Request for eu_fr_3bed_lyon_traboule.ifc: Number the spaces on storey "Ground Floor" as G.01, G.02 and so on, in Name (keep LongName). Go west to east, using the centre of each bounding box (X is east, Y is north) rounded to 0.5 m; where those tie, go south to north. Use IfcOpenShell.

First a look at what the model holds.

```python
import ifcopenshell
import ifcopenshell.util.element
import ifcopenshell.util.placement

model = ifcopenshell.open("eu_fr_3bed_lyon_traboule.ifc")
print(model.schema)
storey = next(s for s in model.by_type("IfcBuildingStorey") if s.Name == "Ground Floor")
spaces = [e for e in ifcopenshell.util.element.get_decomposition(storey) if e.is_a("IfcSpace")]
for e in sorted(spaces, key=lambda e: e.id()):
    origin = ifcopenshell.util.placement.get_local_placement(e.ObjectPlacement)[:3, 3]
    print(e.id(), e.Name, e.LongName, origin.round(2) + 0.0, sep=" | ")
```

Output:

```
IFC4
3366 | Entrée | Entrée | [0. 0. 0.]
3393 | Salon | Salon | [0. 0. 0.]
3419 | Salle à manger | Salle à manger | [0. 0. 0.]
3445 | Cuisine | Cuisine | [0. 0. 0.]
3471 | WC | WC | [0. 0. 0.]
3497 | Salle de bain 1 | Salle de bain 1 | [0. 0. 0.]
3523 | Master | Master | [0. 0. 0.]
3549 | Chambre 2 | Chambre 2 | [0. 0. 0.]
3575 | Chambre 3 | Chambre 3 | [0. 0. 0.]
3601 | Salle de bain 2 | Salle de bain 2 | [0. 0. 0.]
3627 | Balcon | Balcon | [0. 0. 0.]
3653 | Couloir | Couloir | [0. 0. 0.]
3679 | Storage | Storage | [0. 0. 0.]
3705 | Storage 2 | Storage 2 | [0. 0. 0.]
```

```python
import ifcopenshell
import ifcopenshell.geom
import ifcopenshell.util.element
import ifcopenshell.util.shape

model = ifcopenshell.open("eu_fr_3bed_lyon_traboule.ifc")
settings = ifcopenshell.geom.settings()
settings.set("use-world-coords", True)


def centre(element):
    shape = ifcopenshell.geom.create_shape(settings, element)
    return ifcopenshell.util.shape.get_bbox_centroid(shape.geometry)


storey = next(s for s in model.by_type("IfcBuildingStorey") if s.Name == "Ground Floor")
spaces = [e for e in ifcopenshell.util.element.get_decomposition(storey) if e.is_a("IfcSpace")]

# Insertion points can sit at a corner or the storey origin, so sort by the geometry (in metres).
centres = {e: centre(e) for e in spaces}
spaces.sort(key=lambda e: (round(centres[e][0] / 0.5), centres[e][1]))

for i, e in enumerate(spaces, start=1):
    number = f"G.{i:02d}"
    e.Name = number
    print(e.id(), number)

model.write("eu_fr_3bed_lyon_traboule_edited.ifc")
```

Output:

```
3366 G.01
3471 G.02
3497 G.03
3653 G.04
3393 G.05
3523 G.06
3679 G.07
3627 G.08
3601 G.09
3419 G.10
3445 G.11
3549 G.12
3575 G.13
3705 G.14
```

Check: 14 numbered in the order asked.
